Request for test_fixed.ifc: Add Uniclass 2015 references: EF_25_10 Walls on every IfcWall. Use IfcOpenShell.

First a look at what the model holds.

```python
import ifcopenshell

model = ifcopenshell.open("test_fixed.ifc")
print(model.schema)
print("classifications:", [c.Name for c in model.by_type("IfcClassification")])
for ifc_class in ("IfcDoor", "IfcRoof", "IfcStair", "IfcWall", "IfcWindow"):
    print(ifc_class, len(model.by_type(ifc_class)))
```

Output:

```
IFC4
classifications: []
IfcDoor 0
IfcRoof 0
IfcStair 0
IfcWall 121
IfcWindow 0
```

```python
import ifcopenshell
import ifcopenshell.api.classification

model = ifcopenshell.open("test_fixed.ifc")

system = ifcopenshell.api.classification.add_classification(model, classification="Uniclass 2015")

codes = {
    "IfcWall": ("EF_25_10", "Walls"),
}
for ifc_class, (code, name) in codes.items():
    products = model.by_type(ifc_class)
    ifcopenshell.api.classification.add_reference(
        model, products=products, classification=system, identification=code, name=name
    )
    print(code, len(products))

model.write("test_fixed_updated.ifc")
```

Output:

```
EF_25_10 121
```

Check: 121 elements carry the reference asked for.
